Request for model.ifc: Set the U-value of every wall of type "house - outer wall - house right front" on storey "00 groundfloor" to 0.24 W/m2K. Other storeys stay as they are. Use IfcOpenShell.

First a look at what the model holds.

```python
import ifcopenshell
import ifcopenshell.util.element

model = ifcopenshell.open("model.ifc")
print(model.schema)
storey = next(s for s in model.by_type("IfcBuildingStorey") if s.Name == "00 groundfloor")
walls = [e for e in ifcopenshell.util.element.get_decomposition(storey) if e.is_a("IfcWall")]
seen = {}
for e in walls:
    element_type = ifcopenshell.util.element.get_type(e)
    key = (element_type.Name if element_type != e and element_type else None, ifcopenshell.util.element.get_pset(e, "Pset_WallCommon", "ThermalTransmittance"))
    seen[key] = seen.get(key, 0) + 1
for (name, value), count in sorted(seen.items(), key=str):
    print(count, "x", name, "|", value)
```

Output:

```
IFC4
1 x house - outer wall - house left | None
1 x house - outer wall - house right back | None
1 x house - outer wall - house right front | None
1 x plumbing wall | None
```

```python
import ifcopenshell
import ifcopenshell.api.pset
import ifcopenshell.util.element

model = ifcopenshell.open("model.ifc")

storey = next(s for s in model.by_type("IfcBuildingStorey") if s.Name == "00 groundfloor")
walls = [e for e in ifcopenshell.util.element.get_decomposition(storey) if e.is_a("IfcWall")]

count = 0
for e in walls:
    element_type = ifcopenshell.util.element.get_type(e)
    if element_type in (None, e) or element_type.Name != "house - outer wall - house right front":
        continue
    # add_pset returns the element's existing set when there is one.
    pset = ifcopenshell.api.pset.add_pset(model, product=e, name="Pset_WallCommon")
    ifcopenshell.api.pset.edit_pset(model, pset=pset, properties={"ThermalTransmittance": 0.24})
    count += 1

print(count, "walls updated")

model.write("model-out.ifc")
```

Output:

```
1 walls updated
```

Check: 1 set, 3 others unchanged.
